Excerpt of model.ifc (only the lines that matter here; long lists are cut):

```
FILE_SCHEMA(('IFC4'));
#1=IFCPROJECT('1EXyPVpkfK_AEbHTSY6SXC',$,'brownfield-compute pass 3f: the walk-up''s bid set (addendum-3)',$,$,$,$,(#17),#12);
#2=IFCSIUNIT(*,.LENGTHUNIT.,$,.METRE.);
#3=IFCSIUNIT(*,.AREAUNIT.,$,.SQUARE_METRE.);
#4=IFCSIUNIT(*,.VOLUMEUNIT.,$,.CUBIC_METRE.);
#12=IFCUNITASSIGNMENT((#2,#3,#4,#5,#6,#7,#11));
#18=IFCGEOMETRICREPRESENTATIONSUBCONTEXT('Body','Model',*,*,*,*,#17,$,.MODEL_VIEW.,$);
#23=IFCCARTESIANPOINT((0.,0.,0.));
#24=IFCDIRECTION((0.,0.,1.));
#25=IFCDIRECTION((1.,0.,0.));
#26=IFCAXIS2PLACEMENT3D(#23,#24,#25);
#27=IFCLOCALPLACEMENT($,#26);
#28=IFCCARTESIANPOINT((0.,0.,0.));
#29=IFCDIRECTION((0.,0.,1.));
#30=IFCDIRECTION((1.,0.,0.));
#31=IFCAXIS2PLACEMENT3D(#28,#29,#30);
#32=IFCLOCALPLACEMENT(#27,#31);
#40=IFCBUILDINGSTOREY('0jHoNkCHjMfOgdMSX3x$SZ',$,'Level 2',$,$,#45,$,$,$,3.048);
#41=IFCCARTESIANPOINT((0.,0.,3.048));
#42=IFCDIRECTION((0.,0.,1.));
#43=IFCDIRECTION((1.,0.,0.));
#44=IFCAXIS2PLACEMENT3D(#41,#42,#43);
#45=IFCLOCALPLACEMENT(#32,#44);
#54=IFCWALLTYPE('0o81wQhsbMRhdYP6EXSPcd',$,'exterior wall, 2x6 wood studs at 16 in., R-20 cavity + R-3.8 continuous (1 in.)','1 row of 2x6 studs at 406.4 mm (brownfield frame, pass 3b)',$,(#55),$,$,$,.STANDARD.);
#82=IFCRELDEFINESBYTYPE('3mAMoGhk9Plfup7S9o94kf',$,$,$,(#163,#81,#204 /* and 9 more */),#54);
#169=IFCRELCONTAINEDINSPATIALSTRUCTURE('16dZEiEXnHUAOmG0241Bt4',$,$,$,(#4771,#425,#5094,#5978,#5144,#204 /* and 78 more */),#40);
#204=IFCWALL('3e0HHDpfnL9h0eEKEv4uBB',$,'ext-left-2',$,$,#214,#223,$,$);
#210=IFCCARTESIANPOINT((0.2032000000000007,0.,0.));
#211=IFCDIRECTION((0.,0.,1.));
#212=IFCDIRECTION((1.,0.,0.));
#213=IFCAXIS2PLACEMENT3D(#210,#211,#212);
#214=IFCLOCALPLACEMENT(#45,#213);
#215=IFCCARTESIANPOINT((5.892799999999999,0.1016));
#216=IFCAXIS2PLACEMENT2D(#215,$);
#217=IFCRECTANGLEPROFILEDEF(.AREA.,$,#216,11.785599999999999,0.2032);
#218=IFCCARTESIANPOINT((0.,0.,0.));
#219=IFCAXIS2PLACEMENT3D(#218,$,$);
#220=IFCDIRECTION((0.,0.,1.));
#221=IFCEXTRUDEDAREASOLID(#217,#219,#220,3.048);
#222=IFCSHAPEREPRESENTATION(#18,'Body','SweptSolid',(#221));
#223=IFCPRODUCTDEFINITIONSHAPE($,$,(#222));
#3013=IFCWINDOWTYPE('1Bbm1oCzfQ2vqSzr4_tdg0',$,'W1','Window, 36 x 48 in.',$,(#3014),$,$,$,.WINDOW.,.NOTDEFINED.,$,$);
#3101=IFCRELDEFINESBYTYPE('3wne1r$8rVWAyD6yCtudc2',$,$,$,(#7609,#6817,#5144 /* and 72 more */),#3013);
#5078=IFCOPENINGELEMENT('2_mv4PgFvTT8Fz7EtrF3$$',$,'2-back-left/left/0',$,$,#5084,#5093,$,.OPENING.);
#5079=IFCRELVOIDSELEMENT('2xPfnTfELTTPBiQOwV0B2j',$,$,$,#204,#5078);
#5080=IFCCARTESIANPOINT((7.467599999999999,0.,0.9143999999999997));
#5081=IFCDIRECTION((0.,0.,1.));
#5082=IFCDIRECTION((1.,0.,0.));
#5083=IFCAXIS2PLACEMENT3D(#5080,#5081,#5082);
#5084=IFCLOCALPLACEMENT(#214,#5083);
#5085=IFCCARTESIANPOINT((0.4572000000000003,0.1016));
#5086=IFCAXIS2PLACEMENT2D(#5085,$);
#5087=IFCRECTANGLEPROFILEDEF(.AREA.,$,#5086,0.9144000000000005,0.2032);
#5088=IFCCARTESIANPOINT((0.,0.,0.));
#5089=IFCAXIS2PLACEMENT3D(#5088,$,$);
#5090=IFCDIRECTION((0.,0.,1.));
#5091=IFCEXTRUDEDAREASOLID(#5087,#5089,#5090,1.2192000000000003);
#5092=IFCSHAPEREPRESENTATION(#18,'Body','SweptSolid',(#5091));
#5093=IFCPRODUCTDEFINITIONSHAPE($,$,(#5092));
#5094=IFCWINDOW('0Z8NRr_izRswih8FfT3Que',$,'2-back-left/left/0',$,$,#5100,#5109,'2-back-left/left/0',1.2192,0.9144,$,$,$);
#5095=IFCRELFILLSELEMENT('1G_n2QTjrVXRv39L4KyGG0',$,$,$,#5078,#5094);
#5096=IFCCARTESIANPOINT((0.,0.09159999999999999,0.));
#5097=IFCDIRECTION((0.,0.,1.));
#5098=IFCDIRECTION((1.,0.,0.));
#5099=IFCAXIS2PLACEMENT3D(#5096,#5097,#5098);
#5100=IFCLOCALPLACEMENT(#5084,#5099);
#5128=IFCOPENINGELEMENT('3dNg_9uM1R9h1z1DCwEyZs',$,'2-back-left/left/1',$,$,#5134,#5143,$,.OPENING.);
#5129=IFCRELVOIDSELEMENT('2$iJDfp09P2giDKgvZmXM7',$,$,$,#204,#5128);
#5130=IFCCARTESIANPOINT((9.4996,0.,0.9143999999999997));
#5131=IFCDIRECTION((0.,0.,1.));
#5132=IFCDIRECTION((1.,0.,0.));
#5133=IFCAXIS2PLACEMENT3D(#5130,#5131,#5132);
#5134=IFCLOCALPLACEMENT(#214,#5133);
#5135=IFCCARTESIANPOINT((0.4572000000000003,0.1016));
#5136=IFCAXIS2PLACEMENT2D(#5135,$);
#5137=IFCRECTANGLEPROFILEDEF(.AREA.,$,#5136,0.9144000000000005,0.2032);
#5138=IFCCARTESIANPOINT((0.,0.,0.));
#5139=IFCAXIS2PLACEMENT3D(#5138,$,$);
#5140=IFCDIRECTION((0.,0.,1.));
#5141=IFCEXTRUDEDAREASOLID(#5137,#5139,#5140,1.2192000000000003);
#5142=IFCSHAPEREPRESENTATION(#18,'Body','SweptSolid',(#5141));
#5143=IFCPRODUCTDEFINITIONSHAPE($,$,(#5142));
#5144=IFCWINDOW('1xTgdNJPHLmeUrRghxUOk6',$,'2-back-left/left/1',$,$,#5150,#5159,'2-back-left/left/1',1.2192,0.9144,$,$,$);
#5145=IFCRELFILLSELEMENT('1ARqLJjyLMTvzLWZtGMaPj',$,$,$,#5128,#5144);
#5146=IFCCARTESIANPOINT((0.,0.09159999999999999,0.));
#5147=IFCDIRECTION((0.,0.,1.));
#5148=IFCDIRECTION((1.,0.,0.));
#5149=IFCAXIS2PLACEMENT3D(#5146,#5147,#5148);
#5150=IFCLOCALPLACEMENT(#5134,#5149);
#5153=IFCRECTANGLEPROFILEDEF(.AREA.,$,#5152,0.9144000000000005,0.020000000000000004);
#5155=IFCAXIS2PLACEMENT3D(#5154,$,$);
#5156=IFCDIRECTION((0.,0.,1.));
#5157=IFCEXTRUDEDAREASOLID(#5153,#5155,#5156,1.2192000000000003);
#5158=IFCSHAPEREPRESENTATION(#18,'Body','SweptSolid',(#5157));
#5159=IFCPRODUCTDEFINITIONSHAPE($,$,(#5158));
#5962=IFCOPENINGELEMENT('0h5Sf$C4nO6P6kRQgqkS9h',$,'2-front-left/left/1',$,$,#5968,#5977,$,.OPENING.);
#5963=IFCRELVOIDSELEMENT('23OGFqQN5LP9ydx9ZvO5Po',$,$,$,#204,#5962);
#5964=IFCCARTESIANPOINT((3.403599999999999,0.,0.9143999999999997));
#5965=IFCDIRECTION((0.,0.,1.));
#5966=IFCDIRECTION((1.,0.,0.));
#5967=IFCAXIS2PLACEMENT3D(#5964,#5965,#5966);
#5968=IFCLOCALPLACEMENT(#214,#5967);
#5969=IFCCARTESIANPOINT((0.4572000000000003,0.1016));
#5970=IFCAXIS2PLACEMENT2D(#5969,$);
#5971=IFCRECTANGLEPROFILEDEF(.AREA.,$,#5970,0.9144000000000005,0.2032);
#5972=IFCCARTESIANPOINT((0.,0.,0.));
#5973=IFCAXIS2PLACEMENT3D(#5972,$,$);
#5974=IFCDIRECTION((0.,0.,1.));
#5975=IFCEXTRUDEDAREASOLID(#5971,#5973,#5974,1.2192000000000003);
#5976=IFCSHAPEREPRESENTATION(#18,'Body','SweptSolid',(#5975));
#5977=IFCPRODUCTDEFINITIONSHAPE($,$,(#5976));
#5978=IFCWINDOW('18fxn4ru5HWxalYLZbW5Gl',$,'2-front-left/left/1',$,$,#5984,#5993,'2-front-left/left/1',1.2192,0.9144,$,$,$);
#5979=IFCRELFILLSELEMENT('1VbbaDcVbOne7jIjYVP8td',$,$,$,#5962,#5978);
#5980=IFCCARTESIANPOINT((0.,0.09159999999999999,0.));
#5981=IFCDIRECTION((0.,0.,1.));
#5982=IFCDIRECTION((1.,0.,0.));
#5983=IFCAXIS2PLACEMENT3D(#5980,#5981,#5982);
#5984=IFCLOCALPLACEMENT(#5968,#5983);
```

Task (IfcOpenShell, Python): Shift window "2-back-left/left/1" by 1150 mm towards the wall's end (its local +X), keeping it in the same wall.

```python
import ifcopenshell
import ifcopenshell.api.geometry
import ifcopenshell.util.placement

model = ifcopenshell.open("model.ifc")

window = model.by_id(5144)
opening = window.FillsVoids[0].RelatingOpeningElement
wall = opening.VoidsElements[0].RelatingBuildingElement

wall_matrix = ifcopenshell.util.placement.get_local_placement(wall.ObjectPlacement)
shift = wall_matrix[:3, 0] * 1.15
before = ifcopenshell.util.placement.get_local_placement(window.ObjectPlacement)[:3, 3].copy()

# The window is placed relative to its opening, so it follows when the opening moves.
matrix = ifcopenshell.util.placement.get_local_placement(opening.ObjectPlacement)
matrix[:3, 3] += shift
ifcopenshell.api.geometry.edit_object_placement(
    model, product=opening, matrix=matrix, is_si=False, should_transform_children=True
)

after = ifcopenshell.util.placement.get_local_placement(window.ObjectPlacement)[:3, 3]
print("window moved by", (after - before).round(3) + 0.0)

model.write("model-out.ifc")
```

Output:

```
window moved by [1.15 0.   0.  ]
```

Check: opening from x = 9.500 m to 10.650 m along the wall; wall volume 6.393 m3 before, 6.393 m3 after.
